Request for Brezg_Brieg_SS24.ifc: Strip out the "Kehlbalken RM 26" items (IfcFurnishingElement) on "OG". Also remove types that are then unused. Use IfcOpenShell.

First a look at what the model holds.

```python
import ifcopenshell
import ifcopenshell.util.element

model = ifcopenshell.open("Brezg_Brieg_SS24.ifc")
print(model.schema)
storey = next(s for s in model.by_type("IfcBuildingStorey") if s.Name == "OG")
furniture = [e for e in ifcopenshell.util.element.get_decomposition(storey) if e.is_a("IfcFurnishingElement")]
seen = {}
for e in furniture:
    element_type = ifcopenshell.util.element.get_type(e)
    name = element_type.Name if element_type not in (None, e) else None
    seen[name] = seen.get(name, 0) + 1
for name, count in sorted(seen.items(), key=str):
    print(count, "x", name)
```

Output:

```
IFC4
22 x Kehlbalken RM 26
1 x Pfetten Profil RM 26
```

```python
import ifcopenshell
import ifcopenshell.api.root
import ifcopenshell.util.element

model = ifcopenshell.open("Brezg_Brieg_SS24.ifc")

storey = next(s for s in model.by_type("IfcBuildingStorey") if s.Name == "OG")
furniture = [e for e in ifcopenshell.util.element.get_decomposition(storey) if e.is_a("IfcFurnishingElement")]
targets = [e for e in furniture if (t := ifcopenshell.util.element.get_type(e)) not in (None, e) and t.Name == "Kehlbalken RM 26"]
types = {ifcopenshell.util.element.get_type(e) for e in targets} - {None, *targets}

for e in targets:
    ifcopenshell.api.root.remove_product(model, product=e)
print(len(targets), "removed")

unused = [t for t in types if not ifcopenshell.util.element.get_types(t)]
for t in unused:
    ifcopenshell.api.root.remove_product(model, product=t)
print(len(unused), "unused types removed")

model.write("Brezg_Brieg_SS24_updated.ifc")
```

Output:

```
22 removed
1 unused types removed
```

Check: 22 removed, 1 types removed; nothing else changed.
